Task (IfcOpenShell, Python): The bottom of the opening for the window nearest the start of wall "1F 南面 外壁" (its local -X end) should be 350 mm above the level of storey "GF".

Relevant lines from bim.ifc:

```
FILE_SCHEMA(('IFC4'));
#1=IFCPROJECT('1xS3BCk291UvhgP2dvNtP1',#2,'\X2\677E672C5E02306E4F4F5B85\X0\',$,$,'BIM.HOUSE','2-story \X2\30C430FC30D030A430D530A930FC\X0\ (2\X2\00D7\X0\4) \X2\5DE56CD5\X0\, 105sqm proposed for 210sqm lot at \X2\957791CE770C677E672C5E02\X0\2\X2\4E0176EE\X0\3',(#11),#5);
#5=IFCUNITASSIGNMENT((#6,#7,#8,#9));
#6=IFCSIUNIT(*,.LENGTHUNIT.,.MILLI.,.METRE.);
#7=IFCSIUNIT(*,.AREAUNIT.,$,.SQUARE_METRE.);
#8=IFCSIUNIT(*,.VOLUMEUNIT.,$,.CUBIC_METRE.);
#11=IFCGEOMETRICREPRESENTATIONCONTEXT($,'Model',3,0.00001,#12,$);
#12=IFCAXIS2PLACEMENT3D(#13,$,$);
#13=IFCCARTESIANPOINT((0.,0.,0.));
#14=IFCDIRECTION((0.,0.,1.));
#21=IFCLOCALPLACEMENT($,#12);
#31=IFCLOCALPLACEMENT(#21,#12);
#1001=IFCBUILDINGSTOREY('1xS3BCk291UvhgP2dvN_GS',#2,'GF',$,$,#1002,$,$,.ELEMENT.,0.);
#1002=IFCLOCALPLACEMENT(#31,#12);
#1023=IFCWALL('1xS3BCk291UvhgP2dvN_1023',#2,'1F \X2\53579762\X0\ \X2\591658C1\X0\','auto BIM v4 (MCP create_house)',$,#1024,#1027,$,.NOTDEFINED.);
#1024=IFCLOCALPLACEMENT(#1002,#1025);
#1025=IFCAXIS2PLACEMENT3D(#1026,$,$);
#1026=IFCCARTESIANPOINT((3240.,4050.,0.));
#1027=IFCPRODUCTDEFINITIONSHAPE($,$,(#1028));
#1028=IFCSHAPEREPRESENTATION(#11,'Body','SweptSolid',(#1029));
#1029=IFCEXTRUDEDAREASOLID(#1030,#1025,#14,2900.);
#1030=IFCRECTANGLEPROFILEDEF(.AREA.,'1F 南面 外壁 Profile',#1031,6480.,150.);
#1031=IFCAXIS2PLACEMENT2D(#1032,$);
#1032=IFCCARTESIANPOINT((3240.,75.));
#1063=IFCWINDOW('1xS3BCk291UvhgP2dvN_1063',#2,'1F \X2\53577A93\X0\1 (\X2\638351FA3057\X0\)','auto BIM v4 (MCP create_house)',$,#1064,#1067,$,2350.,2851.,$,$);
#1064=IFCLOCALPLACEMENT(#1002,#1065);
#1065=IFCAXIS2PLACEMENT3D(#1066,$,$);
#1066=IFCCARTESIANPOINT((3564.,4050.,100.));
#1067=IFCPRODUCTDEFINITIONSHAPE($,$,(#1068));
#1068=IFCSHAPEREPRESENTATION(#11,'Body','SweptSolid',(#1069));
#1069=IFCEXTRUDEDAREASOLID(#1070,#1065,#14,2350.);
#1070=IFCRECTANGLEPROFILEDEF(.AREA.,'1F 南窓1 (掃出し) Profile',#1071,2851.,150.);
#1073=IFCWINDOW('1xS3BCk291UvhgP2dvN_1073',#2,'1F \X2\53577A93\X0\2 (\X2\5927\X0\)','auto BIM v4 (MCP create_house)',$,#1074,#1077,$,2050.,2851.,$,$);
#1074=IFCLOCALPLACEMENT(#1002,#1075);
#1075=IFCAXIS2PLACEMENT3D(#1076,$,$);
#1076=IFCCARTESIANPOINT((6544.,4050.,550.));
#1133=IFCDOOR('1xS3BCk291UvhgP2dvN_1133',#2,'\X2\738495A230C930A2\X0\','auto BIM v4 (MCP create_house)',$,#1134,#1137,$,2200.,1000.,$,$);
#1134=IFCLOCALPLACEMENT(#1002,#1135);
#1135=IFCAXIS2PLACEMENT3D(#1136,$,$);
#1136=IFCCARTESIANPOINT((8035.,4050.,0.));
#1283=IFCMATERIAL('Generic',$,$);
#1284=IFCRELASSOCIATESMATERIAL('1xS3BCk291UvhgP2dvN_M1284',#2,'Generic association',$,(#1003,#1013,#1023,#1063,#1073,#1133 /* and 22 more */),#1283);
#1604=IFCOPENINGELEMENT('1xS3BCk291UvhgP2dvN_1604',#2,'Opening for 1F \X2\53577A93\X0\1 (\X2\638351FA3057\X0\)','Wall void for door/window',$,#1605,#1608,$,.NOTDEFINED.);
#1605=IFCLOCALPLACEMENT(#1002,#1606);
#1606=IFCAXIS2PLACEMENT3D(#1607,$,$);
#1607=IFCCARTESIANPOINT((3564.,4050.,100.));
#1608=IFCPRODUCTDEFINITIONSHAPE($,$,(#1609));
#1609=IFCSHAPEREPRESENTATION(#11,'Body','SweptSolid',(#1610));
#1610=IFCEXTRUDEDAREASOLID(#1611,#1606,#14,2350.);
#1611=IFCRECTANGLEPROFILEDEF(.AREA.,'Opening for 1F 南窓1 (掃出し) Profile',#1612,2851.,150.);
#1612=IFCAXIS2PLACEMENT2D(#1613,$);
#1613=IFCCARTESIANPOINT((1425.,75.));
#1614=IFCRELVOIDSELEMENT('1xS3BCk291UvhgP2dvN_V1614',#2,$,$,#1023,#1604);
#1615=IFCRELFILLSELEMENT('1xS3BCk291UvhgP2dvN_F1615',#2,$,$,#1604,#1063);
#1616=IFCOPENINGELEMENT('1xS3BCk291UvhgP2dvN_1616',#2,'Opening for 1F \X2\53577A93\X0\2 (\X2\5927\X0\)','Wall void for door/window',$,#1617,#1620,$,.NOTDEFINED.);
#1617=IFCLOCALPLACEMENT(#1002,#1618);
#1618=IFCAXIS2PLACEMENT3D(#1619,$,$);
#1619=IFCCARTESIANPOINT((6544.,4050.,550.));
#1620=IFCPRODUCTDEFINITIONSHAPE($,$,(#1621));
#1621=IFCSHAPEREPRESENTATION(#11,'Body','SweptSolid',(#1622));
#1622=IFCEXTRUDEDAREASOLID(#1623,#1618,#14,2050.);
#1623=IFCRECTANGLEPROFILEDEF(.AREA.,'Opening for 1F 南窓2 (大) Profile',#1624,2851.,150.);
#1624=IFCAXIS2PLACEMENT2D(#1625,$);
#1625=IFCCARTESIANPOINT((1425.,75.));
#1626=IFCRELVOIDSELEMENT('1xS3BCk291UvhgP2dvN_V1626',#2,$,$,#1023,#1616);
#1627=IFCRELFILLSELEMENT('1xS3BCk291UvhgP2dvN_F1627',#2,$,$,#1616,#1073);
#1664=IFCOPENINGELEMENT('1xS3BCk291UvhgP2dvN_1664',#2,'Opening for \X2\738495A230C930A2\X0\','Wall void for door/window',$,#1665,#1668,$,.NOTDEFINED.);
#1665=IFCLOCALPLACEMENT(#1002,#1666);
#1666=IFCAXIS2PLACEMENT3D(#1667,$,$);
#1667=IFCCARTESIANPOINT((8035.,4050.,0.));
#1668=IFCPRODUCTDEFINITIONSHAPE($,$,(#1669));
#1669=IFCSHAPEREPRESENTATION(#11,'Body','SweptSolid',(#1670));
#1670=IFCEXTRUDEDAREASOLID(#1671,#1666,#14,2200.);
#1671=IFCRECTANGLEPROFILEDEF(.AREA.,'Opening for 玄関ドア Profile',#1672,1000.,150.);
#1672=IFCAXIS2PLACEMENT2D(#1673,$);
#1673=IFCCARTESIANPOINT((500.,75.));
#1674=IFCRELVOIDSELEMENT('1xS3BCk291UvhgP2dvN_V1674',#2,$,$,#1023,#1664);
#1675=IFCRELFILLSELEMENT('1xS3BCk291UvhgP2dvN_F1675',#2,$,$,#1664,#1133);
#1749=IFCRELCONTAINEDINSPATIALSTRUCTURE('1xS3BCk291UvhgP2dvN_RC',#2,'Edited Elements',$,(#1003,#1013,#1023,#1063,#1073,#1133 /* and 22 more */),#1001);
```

```python
import numpy as np
import ifcopenshell
import ifcopenshell.api.geometry
import ifcopenshell.geom
import ifcopenshell.util.element
import ifcopenshell.util.placement
import ifcopenshell.util.shape
import ifcopenshell.util.unit

model = ifcopenshell.open("bim.ifc")
unit_scale = ifcopenshell.util.unit.calculate_unit_scale(model)

window = model.by_id(1063)
opening = window.FillsVoids[0].RelatingOpeningElement
storey = ifcopenshell.util.element.get_container(window, ifc_class="IfcBuildingStorey")
level = ifcopenshell.util.placement.get_local_placement(storey.ObjectPlacement)[2, 3]

# The opening's origin need not be at the sill, so measure its lowest point.
shape = ifcopenshell.geom.create_shape(ifcopenshell.geom.settings(), opening)
bottom = ifcopenshell.util.shape.get_shape_bottom_elevation(shape, shape.geometry) / unit_scale
dz = level + 0.35 / unit_scale - bottom

shift = np.array([0.0, 0.0, dz])
# The window is not placed relative to its opening, so move both.
for product in (opening, window):
    matrix = ifcopenshell.util.placement.get_local_placement(product.ObjectPlacement)
    matrix[:3, 3] += shift
    ifcopenshell.api.geometry.edit_object_placement(model, product=product, matrix=matrix, is_si=False)

print(f"moved by {dz * unit_scale:+.3f} m")

model.write("bim_edited.ifc")
```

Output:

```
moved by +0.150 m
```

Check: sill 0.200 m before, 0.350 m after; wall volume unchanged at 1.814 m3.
